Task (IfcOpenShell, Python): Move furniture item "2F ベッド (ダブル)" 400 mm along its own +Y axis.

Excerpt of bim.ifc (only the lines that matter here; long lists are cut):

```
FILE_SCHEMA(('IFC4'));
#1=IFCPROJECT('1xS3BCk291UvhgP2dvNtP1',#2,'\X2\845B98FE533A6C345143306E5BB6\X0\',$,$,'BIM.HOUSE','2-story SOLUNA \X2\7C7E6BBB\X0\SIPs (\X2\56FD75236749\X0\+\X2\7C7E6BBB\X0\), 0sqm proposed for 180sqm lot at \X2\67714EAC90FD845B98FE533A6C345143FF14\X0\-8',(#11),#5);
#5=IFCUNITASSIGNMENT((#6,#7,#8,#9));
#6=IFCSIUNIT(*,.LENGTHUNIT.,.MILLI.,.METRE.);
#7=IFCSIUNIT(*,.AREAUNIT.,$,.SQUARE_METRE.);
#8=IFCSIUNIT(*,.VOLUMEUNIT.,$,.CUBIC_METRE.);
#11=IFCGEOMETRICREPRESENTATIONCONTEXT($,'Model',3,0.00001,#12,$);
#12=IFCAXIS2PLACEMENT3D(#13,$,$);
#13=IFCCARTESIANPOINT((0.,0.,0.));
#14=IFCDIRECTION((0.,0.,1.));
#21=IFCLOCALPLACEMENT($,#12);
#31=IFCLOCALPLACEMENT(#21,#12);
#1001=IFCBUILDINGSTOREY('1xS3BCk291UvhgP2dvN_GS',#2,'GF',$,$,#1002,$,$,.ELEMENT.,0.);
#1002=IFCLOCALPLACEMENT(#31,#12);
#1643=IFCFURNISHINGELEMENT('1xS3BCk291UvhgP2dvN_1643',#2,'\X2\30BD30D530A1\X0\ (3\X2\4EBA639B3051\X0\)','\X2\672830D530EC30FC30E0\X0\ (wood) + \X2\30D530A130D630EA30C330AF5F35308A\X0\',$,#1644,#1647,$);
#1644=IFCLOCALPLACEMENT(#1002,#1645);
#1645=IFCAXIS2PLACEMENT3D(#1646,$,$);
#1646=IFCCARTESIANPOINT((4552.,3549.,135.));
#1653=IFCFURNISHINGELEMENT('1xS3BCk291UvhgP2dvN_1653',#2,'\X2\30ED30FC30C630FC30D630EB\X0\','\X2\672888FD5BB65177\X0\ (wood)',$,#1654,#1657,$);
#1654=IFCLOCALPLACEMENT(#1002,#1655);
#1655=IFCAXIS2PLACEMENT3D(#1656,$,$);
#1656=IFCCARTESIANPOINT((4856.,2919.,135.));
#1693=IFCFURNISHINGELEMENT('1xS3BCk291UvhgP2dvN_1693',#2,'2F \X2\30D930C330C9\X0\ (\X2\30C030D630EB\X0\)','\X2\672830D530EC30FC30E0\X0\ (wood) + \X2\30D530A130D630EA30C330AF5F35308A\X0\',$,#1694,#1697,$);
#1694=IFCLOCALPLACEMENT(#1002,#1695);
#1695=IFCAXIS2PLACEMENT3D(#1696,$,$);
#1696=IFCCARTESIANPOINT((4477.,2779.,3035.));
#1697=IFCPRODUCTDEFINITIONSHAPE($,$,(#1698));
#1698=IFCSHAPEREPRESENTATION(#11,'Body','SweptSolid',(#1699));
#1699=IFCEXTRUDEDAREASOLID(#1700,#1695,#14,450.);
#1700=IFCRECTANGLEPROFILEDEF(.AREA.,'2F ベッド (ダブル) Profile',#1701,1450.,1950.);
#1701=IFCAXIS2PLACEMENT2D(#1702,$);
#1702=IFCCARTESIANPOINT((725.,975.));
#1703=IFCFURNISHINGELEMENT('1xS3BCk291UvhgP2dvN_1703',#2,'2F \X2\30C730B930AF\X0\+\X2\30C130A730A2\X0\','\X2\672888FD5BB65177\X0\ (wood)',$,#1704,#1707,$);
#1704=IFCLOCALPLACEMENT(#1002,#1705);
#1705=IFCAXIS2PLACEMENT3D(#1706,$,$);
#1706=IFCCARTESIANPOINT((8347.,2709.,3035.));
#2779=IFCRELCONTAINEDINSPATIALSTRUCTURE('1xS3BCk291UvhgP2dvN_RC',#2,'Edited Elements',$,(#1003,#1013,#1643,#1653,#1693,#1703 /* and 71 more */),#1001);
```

```python
import ifcopenshell
import ifcopenshell.api.geometry
import ifcopenshell.util.placement
import ifcopenshell.util.unit

model = ifcopenshell.open("bim.ifc")
unit_scale = ifcopenshell.util.unit.calculate_unit_scale(model)

item = model.by_guid("1xS3BCk291UvhgP2dvN_1693")
matrix = ifcopenshell.util.placement.get_local_placement(item.ObjectPlacement)
matrix[:3, 3] += matrix[:3, 1] * 0.4 / unit_scale
ifcopenshell.api.geometry.edit_object_placement(model, product=item, matrix=matrix, is_si=False)

print(ifcopenshell.util.placement.get_local_placement(item.ObjectPlacement).round(3) + 0.0)

model.write("bim_updated.ifc")
```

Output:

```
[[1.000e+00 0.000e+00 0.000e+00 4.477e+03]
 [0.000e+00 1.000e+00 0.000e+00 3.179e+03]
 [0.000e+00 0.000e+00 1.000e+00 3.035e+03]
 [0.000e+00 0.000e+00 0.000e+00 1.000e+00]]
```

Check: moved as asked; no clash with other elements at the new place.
